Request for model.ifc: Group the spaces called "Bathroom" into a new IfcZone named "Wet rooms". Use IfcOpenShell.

First a look at what the model holds.

```python
import ifcopenshell

model = ifcopenshell.open("model.ifc")
print(model.schema)
seen = {}
for space in model.by_type("IfcSpace"):
    seen[space.LongName] = seen.get(space.LongName, 0) + 1
for name, count in sorted(seen.items(), key=str):
    print(count, "x", name)
print("zones:", [z.Name for z in model.by_type("IfcZone")][:20])
```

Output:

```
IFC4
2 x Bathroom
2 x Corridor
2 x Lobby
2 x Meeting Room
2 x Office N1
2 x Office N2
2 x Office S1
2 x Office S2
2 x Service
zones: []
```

```python
import ifcopenshell
import ifcopenshell.api.group
import ifcopenshell.api.root

model = ifcopenshell.open("model.ifc")

names = {"Bathroom"}
spaces = [s for s in model.by_type("IfcSpace") if s.LongName in names]

zone = ifcopenshell.api.root.create_entity(model, ifc_class="IfcZone", name="Wet rooms")
ifcopenshell.api.group.assign_group(model, products=spaces, group=zone)
print(len(spaces), "spaces in", zone.Name)

model.write("model_edited.ifc")
```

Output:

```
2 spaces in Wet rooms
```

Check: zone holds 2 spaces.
